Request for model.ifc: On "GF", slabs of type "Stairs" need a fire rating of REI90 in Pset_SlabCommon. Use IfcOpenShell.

First a look at what the model holds.

```python
import ifcopenshell
import ifcopenshell.util.element

model = ifcopenshell.open("model.ifc")
print(model.schema)
storey = next(s for s in model.by_type("IfcBuildingStorey") if s.Name == "GF")
slabs = [e for e in ifcopenshell.util.element.get_decomposition(storey) if e.is_a("IfcSlab")]
seen = {}
for e in slabs:
    element_type = ifcopenshell.util.element.get_type(e)
    key = (element_type.Name if element_type != e and element_type else None, ifcopenshell.util.element.get_pset(e, "Pset_SlabCommon", "FireRating"))
    seen[key] = seen.get(key, 0) + 1
for (name, value), count in sorted(seen.items(), key=str):
    print(count, "x", name, "|", value)
```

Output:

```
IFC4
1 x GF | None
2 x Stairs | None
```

```python
import ifcopenshell
import ifcopenshell.api.pset
import ifcopenshell.util.element

model = ifcopenshell.open("model.ifc")

storey = next(s for s in model.by_type("IfcBuildingStorey") if s.Name == "GF")
slabs = [e for e in ifcopenshell.util.element.get_decomposition(storey) if e.is_a("IfcSlab")]

count = 0
for e in slabs:
    element_type = ifcopenshell.util.element.get_type(e)
    if element_type in (None, e) or element_type.Name != "Stairs":
        continue
    # add_pset returns the element's existing set when there is one.
    pset = ifcopenshell.api.pset.add_pset(model, product=e, name="Pset_SlabCommon")
    ifcopenshell.api.pset.edit_pset(model, pset=pset, properties={"FireRating": "REI90"})
    count += 1

print(count, "slabs updated")

model.write("model_edited.ifc")
```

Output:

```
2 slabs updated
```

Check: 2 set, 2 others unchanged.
